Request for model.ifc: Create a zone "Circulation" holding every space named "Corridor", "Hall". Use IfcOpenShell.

First a look at what the model holds.

```python
import ifcopenshell

model = ifcopenshell.open("model.ifc")
print(model.schema)
seen = {}
for space in model.by_type("IfcSpace"):
    seen[space.LongName] = seen.get(space.LongName, 0) + 1
for name, count in sorted(seen.items(), key=str):
    print(count, "x", name)
print("zones:", [z.Name for z in model.by_type("IfcZone")][:20])
```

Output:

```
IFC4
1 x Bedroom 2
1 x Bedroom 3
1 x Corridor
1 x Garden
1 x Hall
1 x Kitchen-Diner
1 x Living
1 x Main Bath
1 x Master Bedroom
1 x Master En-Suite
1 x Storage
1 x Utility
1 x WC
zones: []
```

```python
import ifcopenshell
import ifcopenshell.api.group
import ifcopenshell.api.root

model = ifcopenshell.open("model.ifc")

names = {"Corridor", "Hall"}
spaces = [s for s in model.by_type("IfcSpace") if s.LongName in names]

zone = ifcopenshell.api.root.create_entity(model, ifc_class="IfcZone", name="Circulation")
ifcopenshell.api.group.assign_group(model, products=spaces, group=zone)
print(len(spaces), "spaces in", zone.Name)

model.write("model-out.ifc")
```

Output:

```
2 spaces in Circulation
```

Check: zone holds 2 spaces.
